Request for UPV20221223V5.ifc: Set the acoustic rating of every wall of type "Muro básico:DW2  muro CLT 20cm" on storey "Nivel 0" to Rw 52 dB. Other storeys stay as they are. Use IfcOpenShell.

First a look at what the model holds.

```python
import ifcopenshell
import ifcopenshell.util.element

model = ifcopenshell.open("UPV20221223V5.ifc")
print(model.schema)
storey = next(s for s in model.by_type("IfcBuildingStorey") if s.Name == "Nivel 0")
walls = [e for e in ifcopenshell.util.element.get_decomposition(storey) if e.is_a("IfcWall")]
seen = {}
for e in walls:
    element_type = ifcopenshell.util.element.get_type(e)
    key = (element_type.Name if element_type != e and element_type else None, ifcopenshell.util.element.get_pset(e, "Pset_WallCommon", "AcousticRating"))
    seen[key] = seen.get(key, 0) + 1
for (name, value), count in sorted(seen.items(), key=str):
    print(count, "x", name, "|", value)
```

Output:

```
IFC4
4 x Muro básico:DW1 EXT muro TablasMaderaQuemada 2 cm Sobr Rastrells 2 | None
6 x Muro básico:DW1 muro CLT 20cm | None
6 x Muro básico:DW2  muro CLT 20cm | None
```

```python
import ifcopenshell
import ifcopenshell.api.pset
import ifcopenshell.util.element

model = ifcopenshell.open("UPV20221223V5.ifc")

storey = next(s for s in model.by_type("IfcBuildingStorey") if s.Name == "Nivel 0")
walls = [e for e in ifcopenshell.util.element.get_decomposition(storey) if e.is_a("IfcWall")]

count = 0
for e in walls:
    element_type = ifcopenshell.util.element.get_type(e)
    if element_type in (None, e) or element_type.Name != "Muro básico:DW2  muro CLT 20cm":
        continue
    # add_pset returns the element's existing set when there is one.
    pset = ifcopenshell.api.pset.add_pset(model, product=e, name="Pset_WallCommon")
    ifcopenshell.api.pset.edit_pset(model, pset=pset, properties={"AcousticRating": "Rw 52 dB"})
    count += 1

print(count, "walls updated")

model.write("UPV20221223V5_updated.ifc")
```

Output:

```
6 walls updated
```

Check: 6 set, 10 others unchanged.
